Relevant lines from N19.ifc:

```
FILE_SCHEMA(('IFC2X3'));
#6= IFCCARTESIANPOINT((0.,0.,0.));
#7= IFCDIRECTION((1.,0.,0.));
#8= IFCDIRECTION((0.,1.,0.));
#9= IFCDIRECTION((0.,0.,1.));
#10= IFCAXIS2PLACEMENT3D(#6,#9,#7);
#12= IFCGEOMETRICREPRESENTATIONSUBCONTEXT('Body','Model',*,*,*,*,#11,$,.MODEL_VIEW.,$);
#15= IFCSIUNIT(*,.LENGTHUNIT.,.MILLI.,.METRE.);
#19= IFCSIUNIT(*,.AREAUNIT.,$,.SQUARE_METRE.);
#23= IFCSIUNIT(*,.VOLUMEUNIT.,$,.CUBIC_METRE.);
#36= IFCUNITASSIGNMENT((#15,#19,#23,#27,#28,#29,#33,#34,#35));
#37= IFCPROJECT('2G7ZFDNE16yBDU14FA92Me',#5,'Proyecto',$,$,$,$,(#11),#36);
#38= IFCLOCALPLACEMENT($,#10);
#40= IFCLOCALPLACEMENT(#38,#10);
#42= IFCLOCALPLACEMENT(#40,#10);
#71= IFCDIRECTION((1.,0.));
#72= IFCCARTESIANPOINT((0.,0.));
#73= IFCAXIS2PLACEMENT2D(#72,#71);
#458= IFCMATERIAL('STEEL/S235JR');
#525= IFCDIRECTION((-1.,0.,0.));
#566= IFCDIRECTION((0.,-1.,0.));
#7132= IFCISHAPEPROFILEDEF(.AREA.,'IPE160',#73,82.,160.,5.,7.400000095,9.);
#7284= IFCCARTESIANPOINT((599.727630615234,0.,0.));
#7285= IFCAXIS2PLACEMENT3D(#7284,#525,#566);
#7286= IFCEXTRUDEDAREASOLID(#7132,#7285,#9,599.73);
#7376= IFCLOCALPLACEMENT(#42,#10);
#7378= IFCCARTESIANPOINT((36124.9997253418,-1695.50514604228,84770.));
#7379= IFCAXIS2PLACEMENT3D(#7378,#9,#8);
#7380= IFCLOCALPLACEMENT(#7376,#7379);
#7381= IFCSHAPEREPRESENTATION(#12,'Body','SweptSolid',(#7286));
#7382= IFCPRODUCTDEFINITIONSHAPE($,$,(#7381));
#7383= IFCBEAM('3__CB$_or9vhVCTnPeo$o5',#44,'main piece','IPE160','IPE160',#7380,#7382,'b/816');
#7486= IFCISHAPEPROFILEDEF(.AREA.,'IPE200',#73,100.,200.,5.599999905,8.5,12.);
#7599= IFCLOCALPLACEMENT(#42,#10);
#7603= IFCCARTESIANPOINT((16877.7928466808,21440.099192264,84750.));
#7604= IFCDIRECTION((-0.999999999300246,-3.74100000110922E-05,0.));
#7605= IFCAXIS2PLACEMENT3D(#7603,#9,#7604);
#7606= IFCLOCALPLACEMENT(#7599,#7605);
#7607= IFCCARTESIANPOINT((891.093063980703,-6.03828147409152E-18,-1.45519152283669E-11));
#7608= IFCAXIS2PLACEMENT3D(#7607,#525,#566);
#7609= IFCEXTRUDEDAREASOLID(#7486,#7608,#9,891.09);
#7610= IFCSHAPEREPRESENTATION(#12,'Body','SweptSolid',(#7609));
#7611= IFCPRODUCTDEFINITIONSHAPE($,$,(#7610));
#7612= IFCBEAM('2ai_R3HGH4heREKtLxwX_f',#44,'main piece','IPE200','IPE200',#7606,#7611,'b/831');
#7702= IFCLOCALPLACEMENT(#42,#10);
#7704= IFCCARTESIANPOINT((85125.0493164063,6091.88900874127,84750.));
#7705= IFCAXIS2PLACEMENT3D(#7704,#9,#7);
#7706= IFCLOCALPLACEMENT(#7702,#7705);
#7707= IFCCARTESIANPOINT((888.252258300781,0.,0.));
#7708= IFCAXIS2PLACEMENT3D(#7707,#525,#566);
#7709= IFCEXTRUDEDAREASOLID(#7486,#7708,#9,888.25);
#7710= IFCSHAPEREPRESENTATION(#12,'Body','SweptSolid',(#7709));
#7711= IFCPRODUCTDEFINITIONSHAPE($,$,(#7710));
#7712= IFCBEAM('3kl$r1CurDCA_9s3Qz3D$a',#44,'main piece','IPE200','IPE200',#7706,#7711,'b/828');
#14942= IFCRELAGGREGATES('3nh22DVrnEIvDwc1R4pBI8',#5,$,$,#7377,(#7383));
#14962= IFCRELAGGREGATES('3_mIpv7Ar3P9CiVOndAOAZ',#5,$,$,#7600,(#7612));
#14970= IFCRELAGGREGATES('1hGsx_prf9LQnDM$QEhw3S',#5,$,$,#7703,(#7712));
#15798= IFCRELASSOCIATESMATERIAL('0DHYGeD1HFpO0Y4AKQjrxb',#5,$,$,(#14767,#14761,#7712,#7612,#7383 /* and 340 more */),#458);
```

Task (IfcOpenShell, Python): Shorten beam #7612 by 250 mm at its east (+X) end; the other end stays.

```python
import ifcopenshell
import ifcopenshell.util.representation

model = ifcopenshell.open("N19.ifc")

member = model.by_id(7612)
change = -250.0

# The extrusion runs towards the end named, so only its depth changes.
body = ifcopenshell.util.representation.get_representation(member, "Model", "Body")
solid = body.Items[0]
old_length = solid.Depth
solid.Depth += change

print(f"length {old_length:g} -> {solid.Depth:g}")

model.write("N19_v2.ifc")
```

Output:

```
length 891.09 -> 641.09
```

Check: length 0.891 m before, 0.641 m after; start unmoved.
